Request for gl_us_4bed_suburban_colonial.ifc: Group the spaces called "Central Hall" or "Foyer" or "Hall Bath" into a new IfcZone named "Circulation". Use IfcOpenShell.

First a look at what the model holds.

```python
import ifcopenshell

model = ifcopenshell.open("gl_us_4bed_suburban_colonial.ifc")
print(model.schema)
seen = {}
for space in model.by_type("IfcSpace"):
    seen[space.LongName] = seen.get(space.LongName, 0) + 1
for name, count in sorted(seen.items(), key=str):
    print(count, "x", name)
print("zones:", [z.Name for z in model.by_type("IfcZone")][:20])
```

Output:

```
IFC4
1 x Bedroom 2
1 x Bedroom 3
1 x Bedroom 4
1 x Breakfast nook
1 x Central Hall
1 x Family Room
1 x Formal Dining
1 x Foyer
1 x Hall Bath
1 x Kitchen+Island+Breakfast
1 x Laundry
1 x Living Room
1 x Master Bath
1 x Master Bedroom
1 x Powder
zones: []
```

```python
import ifcopenshell
import ifcopenshell.api.group
import ifcopenshell.api.root

model = ifcopenshell.open("gl_us_4bed_suburban_colonial.ifc")

names = {"Central Hall", "Foyer", "Hall Bath"}
spaces = [s for s in model.by_type("IfcSpace") if s.LongName in names]

zone = ifcopenshell.api.root.create_entity(model, ifc_class="IfcZone", name="Circulation")
ifcopenshell.api.group.assign_group(model, products=spaces, group=zone)
print(len(spaces), "spaces in", zone.Name)

model.write("gl_us_4bed_suburban_colonial_updated.ifc")
```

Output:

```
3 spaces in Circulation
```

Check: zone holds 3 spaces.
